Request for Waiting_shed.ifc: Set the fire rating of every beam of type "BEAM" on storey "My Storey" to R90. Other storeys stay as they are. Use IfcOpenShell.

First a look at what the model holds.

```python
import ifcopenshell
import ifcopenshell.util.element

model = ifcopenshell.open("Waiting_shed.ifc")
print(model.schema)
storey = next(s for s in model.by_type("IfcBuildingStorey") if s.Name == "My Storey")
beams = [e for e in ifcopenshell.util.element.get_decomposition(storey) if e.is_a("IfcBeam")]
seen = {}
for e in beams:
    element_type = ifcopenshell.util.element.get_type(e)
    key = (element_type.Name if element_type != e and element_type else None, ifcopenshell.util.element.get_pset(e, "Pset_BeamCommon", "FireRating"))
    seen[key] = seen.get(key, 0) + 1
for (name, value), count in sorted(seen.items(), key=str):
    print(count, "x", name, "|", value)
```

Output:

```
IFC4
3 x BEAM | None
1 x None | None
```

```python
import ifcopenshell
import ifcopenshell.api.pset
import ifcopenshell.util.element

model = ifcopenshell.open("Waiting_shed.ifc")

storey = next(s for s in model.by_type("IfcBuildingStorey") if s.Name == "My Storey")
beams = [e for e in ifcopenshell.util.element.get_decomposition(storey) if e.is_a("IfcBeam")]

count = 0
for e in beams:
    element_type = ifcopenshell.util.element.get_type(e)
    if element_type in (None, e) or element_type.Name != "BEAM":
        continue
    # add_pset returns the element's existing set when there is one.
    pset = ifcopenshell.api.pset.add_pset(model, product=e, name="Pset_BeamCommon")
    ifcopenshell.api.pset.edit_pset(model, pset=pset, properties={"FireRating": "R90"})
    count += 1

print(count, "beams updated")

model.write("Waiting_shed_rev.ifc")
```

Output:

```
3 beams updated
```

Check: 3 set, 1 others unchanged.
